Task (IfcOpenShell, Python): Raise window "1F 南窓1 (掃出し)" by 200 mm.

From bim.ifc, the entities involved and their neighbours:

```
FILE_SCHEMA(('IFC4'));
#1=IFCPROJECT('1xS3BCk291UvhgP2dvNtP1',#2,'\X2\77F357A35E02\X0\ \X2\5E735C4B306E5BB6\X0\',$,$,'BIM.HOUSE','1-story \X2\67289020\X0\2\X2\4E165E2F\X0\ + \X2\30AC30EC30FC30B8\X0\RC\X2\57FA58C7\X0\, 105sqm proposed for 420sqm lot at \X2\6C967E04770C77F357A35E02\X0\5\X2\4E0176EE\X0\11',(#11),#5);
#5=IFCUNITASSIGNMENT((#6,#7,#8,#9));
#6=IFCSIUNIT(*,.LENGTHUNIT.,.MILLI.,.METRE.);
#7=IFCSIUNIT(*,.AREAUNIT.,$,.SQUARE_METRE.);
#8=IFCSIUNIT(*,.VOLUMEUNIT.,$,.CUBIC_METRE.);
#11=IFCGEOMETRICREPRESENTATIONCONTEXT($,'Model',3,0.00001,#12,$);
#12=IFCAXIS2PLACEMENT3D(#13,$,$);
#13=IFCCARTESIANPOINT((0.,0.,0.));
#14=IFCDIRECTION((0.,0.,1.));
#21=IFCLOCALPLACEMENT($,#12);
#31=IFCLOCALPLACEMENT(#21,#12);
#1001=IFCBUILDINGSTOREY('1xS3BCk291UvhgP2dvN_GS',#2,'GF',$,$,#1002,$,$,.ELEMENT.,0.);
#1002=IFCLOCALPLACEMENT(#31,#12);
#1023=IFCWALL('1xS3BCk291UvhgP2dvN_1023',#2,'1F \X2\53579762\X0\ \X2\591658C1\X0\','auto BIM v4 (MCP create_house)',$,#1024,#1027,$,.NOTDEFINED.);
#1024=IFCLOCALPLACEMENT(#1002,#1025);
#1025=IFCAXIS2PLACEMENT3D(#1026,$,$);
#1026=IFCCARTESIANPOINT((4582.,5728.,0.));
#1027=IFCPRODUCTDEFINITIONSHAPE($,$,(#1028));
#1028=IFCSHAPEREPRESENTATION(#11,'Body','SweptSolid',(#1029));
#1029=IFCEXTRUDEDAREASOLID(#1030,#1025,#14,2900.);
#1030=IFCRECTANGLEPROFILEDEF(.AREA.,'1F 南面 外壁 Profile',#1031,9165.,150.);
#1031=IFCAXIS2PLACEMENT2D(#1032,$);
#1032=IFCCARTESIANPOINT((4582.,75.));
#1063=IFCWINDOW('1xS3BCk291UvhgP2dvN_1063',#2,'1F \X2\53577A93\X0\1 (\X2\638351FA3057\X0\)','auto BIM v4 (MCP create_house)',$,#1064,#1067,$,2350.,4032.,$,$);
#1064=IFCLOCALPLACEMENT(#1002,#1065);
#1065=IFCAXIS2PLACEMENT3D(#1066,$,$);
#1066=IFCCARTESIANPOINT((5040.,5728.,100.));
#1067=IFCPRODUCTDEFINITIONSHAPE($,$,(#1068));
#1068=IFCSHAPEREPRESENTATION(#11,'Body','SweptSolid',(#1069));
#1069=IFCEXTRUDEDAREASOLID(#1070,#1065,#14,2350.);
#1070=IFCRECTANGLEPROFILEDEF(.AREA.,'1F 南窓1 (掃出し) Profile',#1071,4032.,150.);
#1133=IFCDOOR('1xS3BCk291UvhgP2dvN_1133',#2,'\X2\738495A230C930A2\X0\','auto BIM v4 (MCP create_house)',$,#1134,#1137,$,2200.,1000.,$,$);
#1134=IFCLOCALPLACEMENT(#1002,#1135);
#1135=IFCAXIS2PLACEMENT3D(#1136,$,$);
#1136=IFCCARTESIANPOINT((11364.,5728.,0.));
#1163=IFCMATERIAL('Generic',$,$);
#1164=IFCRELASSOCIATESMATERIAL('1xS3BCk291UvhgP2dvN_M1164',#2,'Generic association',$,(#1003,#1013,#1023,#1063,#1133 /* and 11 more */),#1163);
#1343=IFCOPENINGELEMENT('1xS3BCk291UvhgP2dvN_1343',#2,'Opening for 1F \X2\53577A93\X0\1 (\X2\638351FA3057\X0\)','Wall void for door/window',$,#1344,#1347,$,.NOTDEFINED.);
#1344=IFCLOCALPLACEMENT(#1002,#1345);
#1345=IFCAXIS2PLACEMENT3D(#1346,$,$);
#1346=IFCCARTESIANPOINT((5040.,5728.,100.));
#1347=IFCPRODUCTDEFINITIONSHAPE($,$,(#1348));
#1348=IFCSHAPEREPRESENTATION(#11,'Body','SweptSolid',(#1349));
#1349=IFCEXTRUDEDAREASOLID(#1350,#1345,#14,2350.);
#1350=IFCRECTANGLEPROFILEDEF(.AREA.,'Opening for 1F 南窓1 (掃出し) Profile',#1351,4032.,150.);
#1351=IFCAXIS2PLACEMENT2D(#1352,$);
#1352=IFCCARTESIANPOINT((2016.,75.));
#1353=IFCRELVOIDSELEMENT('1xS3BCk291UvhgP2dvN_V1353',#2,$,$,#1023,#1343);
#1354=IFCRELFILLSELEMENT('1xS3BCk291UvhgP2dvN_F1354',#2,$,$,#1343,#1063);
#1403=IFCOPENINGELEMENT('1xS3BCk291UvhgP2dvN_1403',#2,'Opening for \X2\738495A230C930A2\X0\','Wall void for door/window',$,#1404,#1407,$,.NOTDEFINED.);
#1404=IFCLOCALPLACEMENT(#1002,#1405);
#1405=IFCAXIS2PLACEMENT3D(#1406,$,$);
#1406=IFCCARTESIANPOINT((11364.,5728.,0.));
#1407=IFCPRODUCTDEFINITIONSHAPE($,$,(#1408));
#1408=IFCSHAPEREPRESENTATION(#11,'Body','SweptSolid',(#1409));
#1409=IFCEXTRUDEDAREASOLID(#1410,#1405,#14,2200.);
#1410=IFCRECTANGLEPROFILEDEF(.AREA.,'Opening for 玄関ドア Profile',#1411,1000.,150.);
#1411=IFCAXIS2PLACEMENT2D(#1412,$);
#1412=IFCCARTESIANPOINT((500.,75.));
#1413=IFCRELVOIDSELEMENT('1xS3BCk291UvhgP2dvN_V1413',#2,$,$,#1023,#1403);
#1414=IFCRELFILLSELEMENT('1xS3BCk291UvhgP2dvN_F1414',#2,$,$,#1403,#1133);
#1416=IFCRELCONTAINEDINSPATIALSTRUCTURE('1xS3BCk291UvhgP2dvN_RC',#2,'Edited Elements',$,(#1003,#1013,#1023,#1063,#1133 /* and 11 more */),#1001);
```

```python
import numpy as np
import ifcopenshell
import ifcopenshell.api.geometry
import ifcopenshell.util.placement
import ifcopenshell.util.unit

model = ifcopenshell.open("bim.ifc")
unit_scale = ifcopenshell.util.unit.calculate_unit_scale(model)

window = model.by_id(1063)
opening = window.FillsVoids[0].RelatingOpeningElement
dz = 200.0

shift = np.array([0.0, 0.0, dz])
# The window is not placed relative to its opening, so move both.
for product in (opening, window):
    matrix = ifcopenshell.util.placement.get_local_placement(product.ObjectPlacement)
    matrix[:3, 3] += shift
    ifcopenshell.api.geometry.edit_object_placement(model, product=product, matrix=matrix, is_si=False)

print(f"moved by {dz * unit_scale:+.3f} m")

model.write("bim_updated.ifc")
```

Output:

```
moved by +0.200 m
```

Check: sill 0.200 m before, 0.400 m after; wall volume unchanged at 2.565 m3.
